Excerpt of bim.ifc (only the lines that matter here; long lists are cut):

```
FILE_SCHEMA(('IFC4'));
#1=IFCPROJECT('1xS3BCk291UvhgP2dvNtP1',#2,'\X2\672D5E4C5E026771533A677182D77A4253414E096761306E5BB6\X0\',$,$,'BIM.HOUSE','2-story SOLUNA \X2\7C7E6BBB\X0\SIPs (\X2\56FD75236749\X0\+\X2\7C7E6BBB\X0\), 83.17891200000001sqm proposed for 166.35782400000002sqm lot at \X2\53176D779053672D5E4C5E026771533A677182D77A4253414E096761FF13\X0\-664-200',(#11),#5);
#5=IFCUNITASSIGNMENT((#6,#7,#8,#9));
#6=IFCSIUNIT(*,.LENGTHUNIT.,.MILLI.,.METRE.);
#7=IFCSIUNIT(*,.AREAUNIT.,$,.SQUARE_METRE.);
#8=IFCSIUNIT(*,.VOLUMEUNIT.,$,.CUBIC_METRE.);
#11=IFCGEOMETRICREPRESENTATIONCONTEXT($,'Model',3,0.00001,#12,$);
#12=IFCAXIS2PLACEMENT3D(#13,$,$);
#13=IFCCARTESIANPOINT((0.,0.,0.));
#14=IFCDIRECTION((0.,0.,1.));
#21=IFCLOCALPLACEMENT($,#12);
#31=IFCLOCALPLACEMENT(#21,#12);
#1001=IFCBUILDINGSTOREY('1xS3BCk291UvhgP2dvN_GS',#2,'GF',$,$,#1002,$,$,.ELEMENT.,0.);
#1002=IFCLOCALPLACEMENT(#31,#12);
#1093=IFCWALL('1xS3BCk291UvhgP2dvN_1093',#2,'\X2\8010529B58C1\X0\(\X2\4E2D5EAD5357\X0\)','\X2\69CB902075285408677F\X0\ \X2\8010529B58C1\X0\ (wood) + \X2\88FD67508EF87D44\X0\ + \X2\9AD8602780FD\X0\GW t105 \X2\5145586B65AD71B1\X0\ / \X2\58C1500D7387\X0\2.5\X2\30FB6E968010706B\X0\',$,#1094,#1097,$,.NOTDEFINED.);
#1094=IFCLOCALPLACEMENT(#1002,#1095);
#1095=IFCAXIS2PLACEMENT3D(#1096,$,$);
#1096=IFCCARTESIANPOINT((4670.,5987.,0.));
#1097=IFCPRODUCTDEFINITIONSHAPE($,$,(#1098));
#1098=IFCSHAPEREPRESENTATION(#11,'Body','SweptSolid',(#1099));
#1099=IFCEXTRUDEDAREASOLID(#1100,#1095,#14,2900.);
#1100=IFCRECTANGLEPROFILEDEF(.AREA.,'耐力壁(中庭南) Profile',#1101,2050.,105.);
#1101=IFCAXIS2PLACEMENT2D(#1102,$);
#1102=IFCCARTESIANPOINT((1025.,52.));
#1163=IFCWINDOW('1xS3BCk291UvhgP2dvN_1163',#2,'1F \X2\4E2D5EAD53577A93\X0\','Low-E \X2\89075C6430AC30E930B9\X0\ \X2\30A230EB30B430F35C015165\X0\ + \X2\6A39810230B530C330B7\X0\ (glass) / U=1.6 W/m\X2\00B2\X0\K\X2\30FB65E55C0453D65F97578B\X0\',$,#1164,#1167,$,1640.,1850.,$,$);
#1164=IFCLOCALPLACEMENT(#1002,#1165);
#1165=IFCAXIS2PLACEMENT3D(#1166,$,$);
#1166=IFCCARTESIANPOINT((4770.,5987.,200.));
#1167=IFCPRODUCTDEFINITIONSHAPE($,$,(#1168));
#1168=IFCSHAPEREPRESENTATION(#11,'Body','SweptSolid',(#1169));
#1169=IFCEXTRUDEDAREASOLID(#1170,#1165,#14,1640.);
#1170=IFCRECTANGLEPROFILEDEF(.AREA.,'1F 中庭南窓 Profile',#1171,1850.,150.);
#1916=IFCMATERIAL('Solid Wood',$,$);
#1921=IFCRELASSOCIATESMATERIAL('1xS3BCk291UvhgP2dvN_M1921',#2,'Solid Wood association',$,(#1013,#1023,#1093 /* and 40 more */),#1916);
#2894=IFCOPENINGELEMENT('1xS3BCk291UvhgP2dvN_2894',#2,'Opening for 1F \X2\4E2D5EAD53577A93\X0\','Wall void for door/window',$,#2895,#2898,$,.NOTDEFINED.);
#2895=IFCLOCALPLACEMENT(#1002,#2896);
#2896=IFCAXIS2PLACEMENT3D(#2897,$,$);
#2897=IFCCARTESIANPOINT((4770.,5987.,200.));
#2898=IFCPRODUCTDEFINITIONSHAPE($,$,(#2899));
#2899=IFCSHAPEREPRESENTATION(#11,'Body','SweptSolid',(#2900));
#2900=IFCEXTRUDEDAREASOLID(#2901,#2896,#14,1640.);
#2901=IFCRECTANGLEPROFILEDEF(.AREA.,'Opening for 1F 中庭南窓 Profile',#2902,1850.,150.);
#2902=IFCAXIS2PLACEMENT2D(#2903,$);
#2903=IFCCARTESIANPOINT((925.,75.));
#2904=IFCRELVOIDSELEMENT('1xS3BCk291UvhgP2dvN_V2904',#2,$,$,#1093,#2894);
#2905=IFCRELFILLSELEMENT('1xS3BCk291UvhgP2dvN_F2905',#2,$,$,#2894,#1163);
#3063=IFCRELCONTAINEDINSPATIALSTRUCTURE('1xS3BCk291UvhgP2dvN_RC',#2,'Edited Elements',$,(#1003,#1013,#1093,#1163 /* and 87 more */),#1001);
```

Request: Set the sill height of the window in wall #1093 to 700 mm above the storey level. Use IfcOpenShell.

```python
import numpy as np
import ifcopenshell
import ifcopenshell.api.geometry
import ifcopenshell.geom
import ifcopenshell.util.element
import ifcopenshell.util.placement
import ifcopenshell.util.shape
import ifcopenshell.util.unit

model = ifcopenshell.open("bim.ifc")
unit_scale = ifcopenshell.util.unit.calculate_unit_scale(model)

window = model.by_guid("1xS3BCk291UvhgP2dvN_1163")
opening = window.FillsVoids[0].RelatingOpeningElement
storey = ifcopenshell.util.element.get_container(window, ifc_class="IfcBuildingStorey")
level = ifcopenshell.util.placement.get_local_placement(storey.ObjectPlacement)[2, 3]

# The opening's origin need not be at the sill, so measure its lowest point.
shape = ifcopenshell.geom.create_shape(ifcopenshell.geom.settings(), opening)
bottom = ifcopenshell.util.shape.get_shape_bottom_elevation(shape, shape.geometry) / unit_scale
dz = level + 0.7 / unit_scale - bottom

shift = np.array([0.0, 0.0, dz])
# The window is not placed relative to its opening, so move both.
for product in (opening, window):
    matrix = ifcopenshell.util.placement.get_local_placement(product.ObjectPlacement)
    matrix[:3, 3] += shift
    ifcopenshell.api.geometry.edit_object_placement(model, product=product, matrix=matrix, is_si=False)

print(f"moved by {dz * unit_scale:+.3f} m")

model.write("bim_rev.ifc")
```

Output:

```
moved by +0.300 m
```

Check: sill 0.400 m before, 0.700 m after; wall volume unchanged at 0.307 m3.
